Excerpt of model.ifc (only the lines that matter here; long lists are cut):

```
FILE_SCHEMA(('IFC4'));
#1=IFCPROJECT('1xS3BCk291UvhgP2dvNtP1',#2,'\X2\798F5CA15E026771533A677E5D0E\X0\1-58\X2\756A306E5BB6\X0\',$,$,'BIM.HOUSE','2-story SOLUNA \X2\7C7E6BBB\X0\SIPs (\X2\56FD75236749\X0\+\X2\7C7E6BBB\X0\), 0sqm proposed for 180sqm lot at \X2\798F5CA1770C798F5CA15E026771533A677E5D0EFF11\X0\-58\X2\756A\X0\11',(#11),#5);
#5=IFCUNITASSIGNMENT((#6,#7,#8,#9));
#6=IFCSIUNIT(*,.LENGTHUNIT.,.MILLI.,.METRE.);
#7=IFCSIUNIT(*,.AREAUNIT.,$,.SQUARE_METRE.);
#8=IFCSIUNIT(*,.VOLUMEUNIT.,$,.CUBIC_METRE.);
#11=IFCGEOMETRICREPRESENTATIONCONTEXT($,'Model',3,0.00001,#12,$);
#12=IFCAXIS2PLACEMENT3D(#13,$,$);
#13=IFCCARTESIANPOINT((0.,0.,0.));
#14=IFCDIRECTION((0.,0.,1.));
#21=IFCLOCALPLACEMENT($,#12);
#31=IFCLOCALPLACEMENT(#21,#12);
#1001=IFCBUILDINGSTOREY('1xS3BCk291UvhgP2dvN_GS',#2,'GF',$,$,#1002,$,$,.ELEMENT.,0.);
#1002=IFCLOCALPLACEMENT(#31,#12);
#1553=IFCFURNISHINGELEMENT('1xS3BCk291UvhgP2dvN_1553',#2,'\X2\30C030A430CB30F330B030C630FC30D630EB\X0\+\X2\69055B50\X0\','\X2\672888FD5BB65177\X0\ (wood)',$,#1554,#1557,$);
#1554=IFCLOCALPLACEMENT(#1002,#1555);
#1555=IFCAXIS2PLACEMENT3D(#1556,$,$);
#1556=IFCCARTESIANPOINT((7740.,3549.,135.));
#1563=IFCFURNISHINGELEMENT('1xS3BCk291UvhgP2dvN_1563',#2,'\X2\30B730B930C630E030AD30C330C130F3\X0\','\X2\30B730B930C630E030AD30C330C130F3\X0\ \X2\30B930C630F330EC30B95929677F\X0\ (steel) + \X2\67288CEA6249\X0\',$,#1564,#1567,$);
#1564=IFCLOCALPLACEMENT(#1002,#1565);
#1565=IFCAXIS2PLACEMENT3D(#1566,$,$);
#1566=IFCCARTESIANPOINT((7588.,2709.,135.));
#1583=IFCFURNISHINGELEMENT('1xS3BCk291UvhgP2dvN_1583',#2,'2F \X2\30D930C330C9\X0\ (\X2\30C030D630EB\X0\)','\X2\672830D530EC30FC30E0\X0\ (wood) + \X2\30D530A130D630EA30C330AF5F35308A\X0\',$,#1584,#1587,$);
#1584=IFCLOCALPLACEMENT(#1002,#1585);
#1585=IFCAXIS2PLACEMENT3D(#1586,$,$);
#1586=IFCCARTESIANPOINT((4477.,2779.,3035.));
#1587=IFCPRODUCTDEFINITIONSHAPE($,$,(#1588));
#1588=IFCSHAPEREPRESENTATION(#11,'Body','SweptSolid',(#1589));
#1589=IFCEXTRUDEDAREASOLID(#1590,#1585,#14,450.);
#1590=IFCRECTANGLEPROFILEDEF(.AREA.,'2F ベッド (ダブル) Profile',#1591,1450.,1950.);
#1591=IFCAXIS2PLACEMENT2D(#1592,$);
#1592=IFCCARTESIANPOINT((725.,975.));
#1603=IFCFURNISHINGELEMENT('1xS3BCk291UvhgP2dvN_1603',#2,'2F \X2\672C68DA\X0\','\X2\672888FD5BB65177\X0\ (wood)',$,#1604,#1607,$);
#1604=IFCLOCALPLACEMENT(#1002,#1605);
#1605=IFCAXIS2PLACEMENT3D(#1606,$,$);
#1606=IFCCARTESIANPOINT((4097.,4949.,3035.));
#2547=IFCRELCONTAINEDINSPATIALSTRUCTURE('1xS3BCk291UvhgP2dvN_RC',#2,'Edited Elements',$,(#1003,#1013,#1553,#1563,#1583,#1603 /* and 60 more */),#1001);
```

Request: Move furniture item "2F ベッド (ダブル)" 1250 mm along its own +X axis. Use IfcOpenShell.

```python
import ifcopenshell
import ifcopenshell.api.geometry
import ifcopenshell.util.placement

model = ifcopenshell.open("model.ifc")

item = model.by_guid("1xS3BCk291UvhgP2dvN_1583")
matrix = ifcopenshell.util.placement.get_local_placement(item.ObjectPlacement)
matrix[:3, 3] += matrix[:3, 0] * 1250.0
ifcopenshell.api.geometry.edit_object_placement(model, product=item, matrix=matrix, is_si=False)

print(ifcopenshell.util.placement.get_local_placement(item.ObjectPlacement).round(3) + 0.0)

model.write("model_edited.ifc")
```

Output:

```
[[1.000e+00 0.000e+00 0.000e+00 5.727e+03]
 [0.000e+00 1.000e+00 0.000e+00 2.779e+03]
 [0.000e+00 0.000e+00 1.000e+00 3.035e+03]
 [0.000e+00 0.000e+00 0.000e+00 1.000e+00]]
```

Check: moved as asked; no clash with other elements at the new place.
